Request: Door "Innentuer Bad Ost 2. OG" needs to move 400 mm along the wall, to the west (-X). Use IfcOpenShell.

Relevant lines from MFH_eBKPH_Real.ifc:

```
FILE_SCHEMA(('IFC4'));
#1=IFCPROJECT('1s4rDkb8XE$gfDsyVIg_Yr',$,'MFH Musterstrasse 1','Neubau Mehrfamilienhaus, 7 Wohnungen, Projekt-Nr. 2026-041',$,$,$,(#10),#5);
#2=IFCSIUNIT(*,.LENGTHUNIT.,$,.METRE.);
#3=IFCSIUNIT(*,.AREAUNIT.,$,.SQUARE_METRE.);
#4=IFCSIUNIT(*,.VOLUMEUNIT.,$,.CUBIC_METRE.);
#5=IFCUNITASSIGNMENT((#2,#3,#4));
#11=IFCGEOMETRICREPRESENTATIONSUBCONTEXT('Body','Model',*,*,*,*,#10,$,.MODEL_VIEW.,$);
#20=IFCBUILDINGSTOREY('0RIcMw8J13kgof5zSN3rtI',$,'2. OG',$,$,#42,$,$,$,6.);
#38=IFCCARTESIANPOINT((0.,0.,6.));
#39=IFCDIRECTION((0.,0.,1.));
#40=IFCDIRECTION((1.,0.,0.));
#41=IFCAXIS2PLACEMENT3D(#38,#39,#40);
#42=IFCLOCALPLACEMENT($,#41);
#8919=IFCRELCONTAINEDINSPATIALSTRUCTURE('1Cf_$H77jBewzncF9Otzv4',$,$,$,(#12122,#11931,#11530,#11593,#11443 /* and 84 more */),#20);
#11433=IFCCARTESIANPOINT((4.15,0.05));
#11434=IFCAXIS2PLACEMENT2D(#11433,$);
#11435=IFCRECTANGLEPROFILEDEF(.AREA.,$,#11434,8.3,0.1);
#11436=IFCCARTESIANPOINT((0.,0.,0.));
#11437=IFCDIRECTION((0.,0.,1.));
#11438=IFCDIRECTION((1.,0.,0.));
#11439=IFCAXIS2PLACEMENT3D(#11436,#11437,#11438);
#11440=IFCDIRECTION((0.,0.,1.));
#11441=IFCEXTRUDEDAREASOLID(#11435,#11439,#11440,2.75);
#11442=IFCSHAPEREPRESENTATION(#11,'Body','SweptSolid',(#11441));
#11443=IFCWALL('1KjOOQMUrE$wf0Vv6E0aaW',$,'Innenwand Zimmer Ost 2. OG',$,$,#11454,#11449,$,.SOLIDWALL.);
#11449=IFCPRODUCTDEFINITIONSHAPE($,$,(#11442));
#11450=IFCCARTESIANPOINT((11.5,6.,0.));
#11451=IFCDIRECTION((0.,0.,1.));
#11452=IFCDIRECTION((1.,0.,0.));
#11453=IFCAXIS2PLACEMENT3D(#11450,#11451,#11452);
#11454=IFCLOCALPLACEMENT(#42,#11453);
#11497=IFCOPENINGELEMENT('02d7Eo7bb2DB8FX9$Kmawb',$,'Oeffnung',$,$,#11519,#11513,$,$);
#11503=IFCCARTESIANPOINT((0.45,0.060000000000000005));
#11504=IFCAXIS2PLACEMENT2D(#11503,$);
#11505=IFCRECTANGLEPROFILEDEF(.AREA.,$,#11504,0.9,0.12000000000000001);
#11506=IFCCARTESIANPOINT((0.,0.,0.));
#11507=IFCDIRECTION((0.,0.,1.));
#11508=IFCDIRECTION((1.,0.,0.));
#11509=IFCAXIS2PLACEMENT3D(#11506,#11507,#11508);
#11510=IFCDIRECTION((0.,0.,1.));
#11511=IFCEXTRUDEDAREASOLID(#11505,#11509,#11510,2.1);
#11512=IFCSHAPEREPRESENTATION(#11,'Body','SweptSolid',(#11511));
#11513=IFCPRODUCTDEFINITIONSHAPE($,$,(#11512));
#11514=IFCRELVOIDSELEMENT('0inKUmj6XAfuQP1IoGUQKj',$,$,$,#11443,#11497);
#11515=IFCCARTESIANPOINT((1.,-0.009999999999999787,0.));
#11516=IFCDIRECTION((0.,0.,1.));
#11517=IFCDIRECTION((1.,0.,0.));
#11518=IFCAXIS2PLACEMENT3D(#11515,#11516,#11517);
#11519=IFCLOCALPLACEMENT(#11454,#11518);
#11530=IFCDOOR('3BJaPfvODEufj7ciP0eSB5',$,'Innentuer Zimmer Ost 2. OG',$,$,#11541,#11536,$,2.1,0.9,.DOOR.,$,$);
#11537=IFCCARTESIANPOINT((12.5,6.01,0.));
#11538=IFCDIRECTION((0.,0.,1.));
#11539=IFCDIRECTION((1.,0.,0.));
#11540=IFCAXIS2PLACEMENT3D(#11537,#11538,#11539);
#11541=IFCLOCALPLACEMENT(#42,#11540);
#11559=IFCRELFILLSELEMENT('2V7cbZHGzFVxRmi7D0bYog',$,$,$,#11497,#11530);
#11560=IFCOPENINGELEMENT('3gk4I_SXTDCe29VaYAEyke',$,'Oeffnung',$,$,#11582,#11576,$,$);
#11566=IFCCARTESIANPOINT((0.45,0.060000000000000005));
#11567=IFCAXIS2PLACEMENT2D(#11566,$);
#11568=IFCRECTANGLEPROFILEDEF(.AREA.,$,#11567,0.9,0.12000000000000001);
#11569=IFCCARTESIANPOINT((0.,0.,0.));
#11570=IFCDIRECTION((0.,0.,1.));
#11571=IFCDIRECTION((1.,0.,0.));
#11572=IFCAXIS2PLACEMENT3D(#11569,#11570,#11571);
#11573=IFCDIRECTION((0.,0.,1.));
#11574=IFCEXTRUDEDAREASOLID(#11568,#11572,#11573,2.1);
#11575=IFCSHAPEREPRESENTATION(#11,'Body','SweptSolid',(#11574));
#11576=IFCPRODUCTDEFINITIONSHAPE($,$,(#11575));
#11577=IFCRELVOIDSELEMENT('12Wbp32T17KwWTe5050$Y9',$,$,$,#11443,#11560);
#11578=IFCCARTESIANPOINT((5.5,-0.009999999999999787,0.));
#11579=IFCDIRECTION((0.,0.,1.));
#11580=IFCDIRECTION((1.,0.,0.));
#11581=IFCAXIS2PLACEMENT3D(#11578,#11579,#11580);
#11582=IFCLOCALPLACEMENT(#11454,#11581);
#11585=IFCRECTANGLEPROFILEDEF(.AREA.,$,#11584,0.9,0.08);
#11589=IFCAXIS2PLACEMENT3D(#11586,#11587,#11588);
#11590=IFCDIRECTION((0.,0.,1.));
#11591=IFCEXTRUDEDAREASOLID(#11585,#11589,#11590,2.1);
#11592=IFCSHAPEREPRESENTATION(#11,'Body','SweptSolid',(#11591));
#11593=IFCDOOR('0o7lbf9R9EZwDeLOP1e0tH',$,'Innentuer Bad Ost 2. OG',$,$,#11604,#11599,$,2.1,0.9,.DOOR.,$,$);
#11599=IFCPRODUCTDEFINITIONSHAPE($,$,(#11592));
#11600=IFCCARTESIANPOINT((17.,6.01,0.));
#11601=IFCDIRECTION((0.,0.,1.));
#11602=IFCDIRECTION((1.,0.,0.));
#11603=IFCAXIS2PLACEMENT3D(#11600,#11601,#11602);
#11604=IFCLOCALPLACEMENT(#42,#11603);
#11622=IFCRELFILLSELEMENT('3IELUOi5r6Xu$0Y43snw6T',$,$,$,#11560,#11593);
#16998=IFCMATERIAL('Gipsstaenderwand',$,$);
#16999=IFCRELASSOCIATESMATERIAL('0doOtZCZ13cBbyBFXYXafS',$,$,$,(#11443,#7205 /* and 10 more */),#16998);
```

```python
import ifcopenshell
import ifcopenshell.api.geometry
import ifcopenshell.util.placement

model = ifcopenshell.open("MFH_eBKPH_Real.ifc")

door = model.by_id(11593)
opening = door.FillsVoids[0].RelatingOpeningElement
wall = opening.VoidsElements[0].RelatingBuildingElement

wall_matrix = ifcopenshell.util.placement.get_local_placement(wall.ObjectPlacement)
shift = wall_matrix[:3, 0] * -0.4
before = ifcopenshell.util.placement.get_local_placement(door.ObjectPlacement)[:3, 3].copy()

# The door is not placed relative to its opening, so move both.
for product in (opening, door):
    matrix = ifcopenshell.util.placement.get_local_placement(product.ObjectPlacement)
    matrix[:3, 3] += shift
    ifcopenshell.api.geometry.edit_object_placement(model, product=product, matrix=matrix, is_si=False)

after = ifcopenshell.util.placement.get_local_placement(door.ObjectPlacement)[:3, 3]
print("door moved by", (after - before).round(3) + 0.0)

model.write("MFH_eBKPH_Real-out.ifc")
```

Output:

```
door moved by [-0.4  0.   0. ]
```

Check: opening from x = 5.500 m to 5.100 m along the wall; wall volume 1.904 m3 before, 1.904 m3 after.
